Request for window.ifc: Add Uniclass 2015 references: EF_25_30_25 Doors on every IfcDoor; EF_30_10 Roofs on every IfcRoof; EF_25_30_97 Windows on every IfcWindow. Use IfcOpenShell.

First a look at what the model holds.

```python
import ifcopenshell

model = ifcopenshell.open("window.ifc")
print(model.schema)
print("classifications:", [c.Name for c in model.by_type("IfcClassification")])
for ifc_class in ("IfcDoor", "IfcRoof", "IfcStair", "IfcWall", "IfcWindow"):
    print(ifc_class, len(model.by_type(ifc_class)))
```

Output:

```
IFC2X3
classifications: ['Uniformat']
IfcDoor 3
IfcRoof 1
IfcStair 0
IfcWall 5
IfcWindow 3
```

```python
import ifcopenshell
import ifcopenshell.api.classification

model = ifcopenshell.open("window.ifc")

# IFC2X3 requires Source and Edition and has no link from the project to the system.
system = model.create_entity("IfcClassification", Source="NBS", Edition="2015", Name="Uniclass 2015")

codes = {
    "IfcDoor": ("EF_25_30_25", "Doors"),
    "IfcRoof": ("EF_30_10", "Roofs"),
    "IfcWindow": ("EF_25_30_97", "Windows"),
}
for ifc_class, (code, name) in codes.items():
    products = model.by_type(ifc_class)
    ifcopenshell.api.classification.add_reference(
        model, products=products, classification=system, identification=code, name=name
    )
    print(code, len(products))

model.write("window_rev.ifc")
```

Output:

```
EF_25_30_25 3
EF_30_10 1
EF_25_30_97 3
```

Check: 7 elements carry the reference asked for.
